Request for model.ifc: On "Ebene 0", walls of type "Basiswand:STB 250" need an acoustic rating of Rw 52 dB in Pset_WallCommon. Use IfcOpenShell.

First a look at what the model holds.

```python
import ifcopenshell
import ifcopenshell.util.element

model = ifcopenshell.open("model.ifc")
print(model.schema)
storey = next(s for s in model.by_type("IfcBuildingStorey") if s.Name == "Ebene 0")
walls = [e for e in ifcopenshell.util.element.get_decomposition(storey) if e.is_a("IfcWall")]
seen = {}
for e in walls:
    element_type = ifcopenshell.util.element.get_type(e)
    key = (element_type.Name if element_type != e and element_type else None, ifcopenshell.util.element.get_pset(e, "Pset_WallCommon", "AcousticRating"))
    seen[key] = seen.get(key, 0) + 1
for (name, value), count in sorted(seen.items(), key=str):
    print(count, "x", name, "|", value)
```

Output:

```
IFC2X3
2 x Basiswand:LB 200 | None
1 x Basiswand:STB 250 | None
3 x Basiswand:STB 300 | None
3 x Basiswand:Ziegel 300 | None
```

```python
import ifcopenshell
import ifcopenshell.api.pset
import ifcopenshell.util.element

model = ifcopenshell.open("model.ifc")

storey = next(s for s in model.by_type("IfcBuildingStorey") if s.Name == "Ebene 0")
walls = [e for e in ifcopenshell.util.element.get_decomposition(storey) if e.is_a("IfcWall")]

count = 0
for e in walls:
    element_type = ifcopenshell.util.element.get_type(e)
    if element_type in (None, e) or element_type.Name != "Basiswand:STB 250":
        continue
    # add_pset returns the element's existing set when there is one.
    pset = ifcopenshell.api.pset.add_pset(model, product=e, name="Pset_WallCommon")
    ifcopenshell.api.pset.edit_pset(model, pset=pset, properties={"AcousticRating": "Rw 52 dB"})
    count += 1

print(count, "walls updated")

model.write("model_updated.ifc")
```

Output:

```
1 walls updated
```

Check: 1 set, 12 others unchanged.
